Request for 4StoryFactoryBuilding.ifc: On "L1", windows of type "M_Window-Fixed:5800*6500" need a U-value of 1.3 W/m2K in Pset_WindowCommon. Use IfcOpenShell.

First a look at what the model holds.

```python
import ifcopenshell
import ifcopenshell.util.element

model = ifcopenshell.open("4StoryFactoryBuilding.ifc")
print(model.schema)
storey = next(s for s in model.by_type("IfcBuildingStorey") if s.Name == "L1")
windows = [e for e in ifcopenshell.util.element.get_decomposition(storey) if e.is_a("IfcWindow")]
seen = {}
for e in windows:
    element_type = ifcopenshell.util.element.get_type(e)
    key = (element_type.Name if element_type != e and element_type else None, ifcopenshell.util.element.get_pset(e, "Pset_WindowCommon", "ThermalTransmittance"))
    seen[key] = seen.get(key, 0) + 1
for (name, value), count in sorted(seen.items(), key=str):
    print(count, "x", name, "|", value)
```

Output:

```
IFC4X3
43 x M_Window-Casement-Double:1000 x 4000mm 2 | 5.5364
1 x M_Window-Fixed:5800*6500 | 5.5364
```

```python
import ifcopenshell
import ifcopenshell.api.pset
import ifcopenshell.util.element

model = ifcopenshell.open("4StoryFactoryBuilding.ifc")

storey = next(s for s in model.by_type("IfcBuildingStorey") if s.Name == "L1")
windows = [e for e in ifcopenshell.util.element.get_decomposition(storey) if e.is_a("IfcWindow")]

count = 0
for e in windows:
    element_type = ifcopenshell.util.element.get_type(e)
    if element_type in (None, e) or element_type.Name != "M_Window-Fixed:5800*6500":
        continue
    # add_pset returns the element's existing set when there is one.
    pset = ifcopenshell.api.pset.add_pset(model, product=e, name="Pset_WindowCommon")
    ifcopenshell.api.pset.edit_pset(model, pset=pset, properties={"ThermalTransmittance": 1.3})
    count += 1

print(count, "windows updated")

model.write("4StoryFactoryBuilding_v2.ifc")
```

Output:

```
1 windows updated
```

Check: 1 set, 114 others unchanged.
